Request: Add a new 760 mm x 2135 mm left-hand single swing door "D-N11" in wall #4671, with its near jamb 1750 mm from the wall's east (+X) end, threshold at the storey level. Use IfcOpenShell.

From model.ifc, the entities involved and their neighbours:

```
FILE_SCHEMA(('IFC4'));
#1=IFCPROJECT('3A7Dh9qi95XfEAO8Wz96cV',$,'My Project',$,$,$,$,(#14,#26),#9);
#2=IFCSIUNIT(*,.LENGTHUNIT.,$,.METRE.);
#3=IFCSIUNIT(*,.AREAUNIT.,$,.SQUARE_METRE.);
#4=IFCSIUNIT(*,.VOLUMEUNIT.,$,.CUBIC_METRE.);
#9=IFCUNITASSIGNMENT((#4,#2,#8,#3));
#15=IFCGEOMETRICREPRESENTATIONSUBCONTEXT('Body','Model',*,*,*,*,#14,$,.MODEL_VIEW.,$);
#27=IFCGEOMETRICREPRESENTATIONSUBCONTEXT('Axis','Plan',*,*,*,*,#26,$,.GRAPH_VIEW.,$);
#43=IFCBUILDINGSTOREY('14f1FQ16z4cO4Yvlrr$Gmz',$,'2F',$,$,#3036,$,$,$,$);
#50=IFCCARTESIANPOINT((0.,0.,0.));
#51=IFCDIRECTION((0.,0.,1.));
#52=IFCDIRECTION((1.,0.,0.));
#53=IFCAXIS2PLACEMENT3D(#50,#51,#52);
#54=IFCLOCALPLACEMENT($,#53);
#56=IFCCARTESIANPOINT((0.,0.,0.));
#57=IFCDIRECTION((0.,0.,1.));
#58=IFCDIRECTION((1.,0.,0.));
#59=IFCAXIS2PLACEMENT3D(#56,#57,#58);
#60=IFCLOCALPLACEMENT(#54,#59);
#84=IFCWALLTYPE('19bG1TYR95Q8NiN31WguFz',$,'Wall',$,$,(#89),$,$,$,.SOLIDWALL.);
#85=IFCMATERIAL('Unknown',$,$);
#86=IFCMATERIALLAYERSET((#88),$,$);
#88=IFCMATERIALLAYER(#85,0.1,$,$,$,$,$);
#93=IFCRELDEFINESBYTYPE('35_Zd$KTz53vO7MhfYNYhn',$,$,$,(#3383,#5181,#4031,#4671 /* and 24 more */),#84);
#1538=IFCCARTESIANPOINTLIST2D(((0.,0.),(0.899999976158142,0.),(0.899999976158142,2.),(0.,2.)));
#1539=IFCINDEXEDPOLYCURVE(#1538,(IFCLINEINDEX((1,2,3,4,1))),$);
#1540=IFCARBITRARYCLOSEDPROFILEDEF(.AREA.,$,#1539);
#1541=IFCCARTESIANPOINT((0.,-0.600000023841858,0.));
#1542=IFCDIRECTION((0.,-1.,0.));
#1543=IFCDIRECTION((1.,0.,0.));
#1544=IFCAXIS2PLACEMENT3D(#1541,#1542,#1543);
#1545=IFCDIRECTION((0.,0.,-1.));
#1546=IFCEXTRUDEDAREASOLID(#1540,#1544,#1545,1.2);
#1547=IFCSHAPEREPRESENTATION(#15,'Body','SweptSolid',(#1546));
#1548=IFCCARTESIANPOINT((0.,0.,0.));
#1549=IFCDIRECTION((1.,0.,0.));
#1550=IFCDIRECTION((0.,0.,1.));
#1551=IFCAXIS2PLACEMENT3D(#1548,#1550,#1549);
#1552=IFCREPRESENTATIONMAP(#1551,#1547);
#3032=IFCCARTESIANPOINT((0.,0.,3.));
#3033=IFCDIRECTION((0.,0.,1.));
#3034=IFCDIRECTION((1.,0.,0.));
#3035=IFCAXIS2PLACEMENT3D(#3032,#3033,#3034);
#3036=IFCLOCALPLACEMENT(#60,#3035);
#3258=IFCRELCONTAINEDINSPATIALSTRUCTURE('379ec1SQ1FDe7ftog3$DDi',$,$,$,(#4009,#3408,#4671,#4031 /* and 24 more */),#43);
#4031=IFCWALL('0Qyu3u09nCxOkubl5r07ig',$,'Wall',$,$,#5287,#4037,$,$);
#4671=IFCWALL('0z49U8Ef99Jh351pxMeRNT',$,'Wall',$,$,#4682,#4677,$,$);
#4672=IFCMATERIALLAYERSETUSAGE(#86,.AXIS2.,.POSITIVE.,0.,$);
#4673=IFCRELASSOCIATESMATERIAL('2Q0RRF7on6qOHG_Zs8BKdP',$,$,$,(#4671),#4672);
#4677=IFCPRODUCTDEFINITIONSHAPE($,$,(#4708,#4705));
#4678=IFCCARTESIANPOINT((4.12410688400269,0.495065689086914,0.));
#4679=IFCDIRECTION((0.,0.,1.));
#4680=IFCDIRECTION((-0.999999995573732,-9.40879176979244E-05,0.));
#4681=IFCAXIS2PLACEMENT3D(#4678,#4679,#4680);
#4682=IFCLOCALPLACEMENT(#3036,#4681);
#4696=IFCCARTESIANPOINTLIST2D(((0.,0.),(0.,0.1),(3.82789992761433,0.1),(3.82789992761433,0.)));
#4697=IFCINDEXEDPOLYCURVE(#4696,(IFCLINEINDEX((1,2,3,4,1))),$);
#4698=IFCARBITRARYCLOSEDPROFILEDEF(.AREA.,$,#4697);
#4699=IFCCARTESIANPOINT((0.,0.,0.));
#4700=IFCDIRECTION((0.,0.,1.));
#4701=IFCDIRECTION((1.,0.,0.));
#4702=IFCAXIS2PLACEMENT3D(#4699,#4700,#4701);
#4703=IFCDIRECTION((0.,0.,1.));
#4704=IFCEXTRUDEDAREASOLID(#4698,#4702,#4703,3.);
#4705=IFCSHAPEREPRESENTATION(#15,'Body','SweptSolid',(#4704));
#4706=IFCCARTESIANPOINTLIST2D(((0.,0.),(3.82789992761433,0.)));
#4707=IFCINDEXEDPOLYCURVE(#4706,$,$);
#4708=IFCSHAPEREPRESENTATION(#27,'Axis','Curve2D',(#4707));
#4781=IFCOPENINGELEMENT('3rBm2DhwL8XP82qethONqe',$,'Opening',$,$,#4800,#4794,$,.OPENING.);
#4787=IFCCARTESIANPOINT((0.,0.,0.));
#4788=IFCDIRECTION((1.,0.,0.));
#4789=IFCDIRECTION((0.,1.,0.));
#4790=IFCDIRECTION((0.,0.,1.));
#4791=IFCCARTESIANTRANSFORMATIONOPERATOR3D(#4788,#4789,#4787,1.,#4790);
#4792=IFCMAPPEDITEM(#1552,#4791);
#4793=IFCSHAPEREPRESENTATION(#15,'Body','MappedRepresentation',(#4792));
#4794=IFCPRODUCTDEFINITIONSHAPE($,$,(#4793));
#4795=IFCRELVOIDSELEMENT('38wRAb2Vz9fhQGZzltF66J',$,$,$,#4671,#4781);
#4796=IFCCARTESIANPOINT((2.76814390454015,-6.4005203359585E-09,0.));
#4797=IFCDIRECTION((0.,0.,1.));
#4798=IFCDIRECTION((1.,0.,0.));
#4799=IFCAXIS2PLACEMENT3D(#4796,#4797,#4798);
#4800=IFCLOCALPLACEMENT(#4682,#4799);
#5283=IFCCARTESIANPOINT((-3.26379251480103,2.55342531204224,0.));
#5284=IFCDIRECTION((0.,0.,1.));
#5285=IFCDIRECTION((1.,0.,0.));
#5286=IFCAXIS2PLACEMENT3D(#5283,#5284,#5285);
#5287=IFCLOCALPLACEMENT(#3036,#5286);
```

```python
import numpy as np
import ifcopenshell
import ifcopenshell.api.feature
import ifcopenshell.api.geometry
import ifcopenshell.api.root
import ifcopenshell.api.spatial
import ifcopenshell.geom
import ifcopenshell.util.element
import ifcopenshell.util.placement
import ifcopenshell.util.representation
import ifcopenshell.util.shape
import ifcopenshell.util.unit

model = ifcopenshell.open("model.ifc")
unit_scale = ifcopenshell.util.unit.calculate_unit_scale(model)
settings = ifcopenshell.geom.settings()


def volume(element):
    """Net volume in cubic metres, openings subtracted."""
    shape = ifcopenshell.geom.create_shape(settings, element)
    return ifcopenshell.util.shape.get_volume(shape.geometry)


wall = model.by_id(4671)
storey = ifcopenshell.util.element.get_container(wall, ifc_class="IfcBuildingStorey")
context = ifcopenshell.util.representation.get_context(model, "Model", "Body", "MODEL_VIEW")
before = volume(wall)

width, height, from_end, sill = 0.76, 2.135, 1.75, 0.0  # metres

# The wall runs along its own X axis, and the end named is its -X end.
wall_shape = ifcopenshell.geom.create_shape(settings, wall)
x, y, z = ifcopenshell.util.shape.get_vertices(wall_shape.geometry).T
start = x.min() + from_end
face, thickness = float(y.min()), float(y.max() - y.min())
wall_matrix = ifcopenshell.util.placement.get_local_placement(wall.ObjectPlacement)
level = ifcopenshell.util.placement.get_local_placement(storey.ObjectPlacement)[2, 3]


def in_wall(x, y):
    """Placement at x, y metres in the wall's axes, at sill height."""
    matrix = wall_matrix.copy()
    matrix[:, 3] = wall_matrix @ np.array([x / unit_scale, y / unit_scale, 0.0, 1.0])
    matrix[2, 3] = level + sill / unit_scale
    return matrix


# Opening: a box that overshoots both wall faces by 50 mm.
opening = ifcopenshell.api.root.create_entity(model, ifc_class="IfcOpeningElement", predefined_type="OPENING")
box = ifcopenshell.api.geometry.add_wall_representation(
    model, context=context, length=width, height=height, thickness=thickness + 0.1
)
ifcopenshell.api.geometry.assign_representation(model, product=opening, representation=box)
ifcopenshell.api.geometry.edit_object_placement(model, product=opening, matrix=in_wall(start, face - 0.05), is_si=False)
ifcopenshell.api.feature.add_feature(model, feature=opening, element=wall)

door = ifcopenshell.api.root.create_entity(model, ifc_class="IfcDoor", name="D-N11", predefined_type="DOOR")
door.OverallWidth, door.OverallHeight = width / unit_scale, height / unit_scale
door.OperationType = "SINGLE_SWING_LEFT"
body = ifcopenshell.api.geometry.add_door_representation(
    model,
    context=context,
    overall_width=door.OverallWidth,
    overall_height=door.OverallHeight,
    operation_type="SINGLE_SWING_LEFT",
    lining_properties={"LiningDepth": thickness / unit_scale, "ThresholdDepth": thickness / unit_scale},
)
ifcopenshell.api.geometry.assign_representation(model, product=door, representation=body)
ifcopenshell.api.spatial.assign_container(model, products=[door], relating_structure=storey)
ifcopenshell.api.feature.add_filling(model, opening=opening, element=door)

# The lining spans the wall, so the door starts at the wall face.
ifcopenshell.api.geometry.edit_object_placement(model, product=door, matrix=in_wall(start, face), is_si=False)

after = volume(wall)

print(f"wall volume {before:.3f} -> {after:.3f} m3")

model.write("model_updated.ifc")
```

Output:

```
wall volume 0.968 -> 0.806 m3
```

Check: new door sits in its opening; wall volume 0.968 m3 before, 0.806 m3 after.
